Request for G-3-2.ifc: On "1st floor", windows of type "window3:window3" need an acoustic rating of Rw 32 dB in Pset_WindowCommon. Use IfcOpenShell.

First a look at what the model holds.

```python
import ifcopenshell
import ifcopenshell.util.element

model = ifcopenshell.open("G-3-2.ifc")
print(model.schema)
storey = next(s for s in model.by_type("IfcBuildingStorey") if s.Name == "1st floor")
windows = [e for e in ifcopenshell.util.element.get_decomposition(storey) if e.is_a("IfcWindow")]
seen = {}
for e in windows:
    element_type = ifcopenshell.util.element.get_type(e)
    key = (element_type.Name if element_type != e and element_type else None, ifcopenshell.util.element.get_pset(e, "Pset_WindowCommon", "AcousticRating"))
    seen[key] = seen.get(key, 0) + 1
for (name, value), count in sorted(seen.items(), key=str):
    print(count, "x", name, "|", value)
```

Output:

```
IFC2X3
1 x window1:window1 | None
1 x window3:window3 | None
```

```python
import ifcopenshell
import ifcopenshell.api.pset
import ifcopenshell.util.element

model = ifcopenshell.open("G-3-2.ifc")

storey = next(s for s in model.by_type("IfcBuildingStorey") if s.Name == "1st floor")
windows = [e for e in ifcopenshell.util.element.get_decomposition(storey) if e.is_a("IfcWindow")]

count = 0
for e in windows:
    element_type = ifcopenshell.util.element.get_type(e)
    if element_type in (None, e) or element_type.Name != "window3:window3":
        continue
    # add_pset returns the element's existing set when there is one.
    pset = ifcopenshell.api.pset.add_pset(model, product=e, name="Pset_WindowCommon")
    ifcopenshell.api.pset.edit_pset(model, pset=pset, properties={"AcousticRating": "Rw 32 dB"})
    count += 1

print(count, "windows updated")

model.write("G-3-2_rev.ifc")
```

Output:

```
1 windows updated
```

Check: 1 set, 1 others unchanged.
